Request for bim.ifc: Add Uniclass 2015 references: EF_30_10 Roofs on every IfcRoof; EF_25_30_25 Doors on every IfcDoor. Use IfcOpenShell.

First a look at what the model holds.

```python
import ifcopenshell

model = ifcopenshell.open("bim.ifc")
print(model.schema)
print("classifications:", [c.Name for c in model.by_type("IfcClassification")])
for ifc_class in ("IfcDoor", "IfcRoof", "IfcStair", "IfcWall", "IfcWindow"):
    print(ifc_class, len(model.by_type(ifc_class)))
```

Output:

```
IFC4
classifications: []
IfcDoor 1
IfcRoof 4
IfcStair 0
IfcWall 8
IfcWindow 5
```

```python
import ifcopenshell
import ifcopenshell.api.classification

model = ifcopenshell.open("bim.ifc")

system = ifcopenshell.api.classification.add_classification(model, classification="Uniclass 2015")

codes = {
    "IfcRoof": ("EF_30_10", "Roofs"),
    "IfcDoor": ("EF_25_30_25", "Doors"),
}
for ifc_class, (code, name) in codes.items():
    products = model.by_type(ifc_class)
    ifcopenshell.api.classification.add_reference(
        model, products=products, classification=system, identification=code, name=name
    )
    print(code, len(products))

model.write("bim_updated.ifc")
```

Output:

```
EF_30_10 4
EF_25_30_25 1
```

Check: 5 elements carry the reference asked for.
